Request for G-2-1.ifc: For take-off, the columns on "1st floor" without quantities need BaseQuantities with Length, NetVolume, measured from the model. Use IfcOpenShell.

First a look at what the model holds.

```python
import ifcopenshell
import ifcopenshell.util.element
import ifcopenshell.util.unit

model = ifcopenshell.open("G-2-1.ifc")
print(model.schema)
for unit_type in ("LENGTHUNIT", "AREAUNIT", "VOLUMEUNIT"):
    print(unit_type, ifcopenshell.util.unit.calculate_unit_scale(model, unit_type))
storey = next(s for s in model.by_type("IfcBuildingStorey") if s.Name == "1st floor")
columns = [e for e in ifcopenshell.util.element.get_decomposition(storey) if e.is_a("IfcColumn")]
for e in sorted(columns, key=lambda e: e.id()):
    print(e.id(), e.is_a(), e.Name, list(ifcopenshell.util.element.get_psets(e, qtos_only=True)), sep=" | ")
```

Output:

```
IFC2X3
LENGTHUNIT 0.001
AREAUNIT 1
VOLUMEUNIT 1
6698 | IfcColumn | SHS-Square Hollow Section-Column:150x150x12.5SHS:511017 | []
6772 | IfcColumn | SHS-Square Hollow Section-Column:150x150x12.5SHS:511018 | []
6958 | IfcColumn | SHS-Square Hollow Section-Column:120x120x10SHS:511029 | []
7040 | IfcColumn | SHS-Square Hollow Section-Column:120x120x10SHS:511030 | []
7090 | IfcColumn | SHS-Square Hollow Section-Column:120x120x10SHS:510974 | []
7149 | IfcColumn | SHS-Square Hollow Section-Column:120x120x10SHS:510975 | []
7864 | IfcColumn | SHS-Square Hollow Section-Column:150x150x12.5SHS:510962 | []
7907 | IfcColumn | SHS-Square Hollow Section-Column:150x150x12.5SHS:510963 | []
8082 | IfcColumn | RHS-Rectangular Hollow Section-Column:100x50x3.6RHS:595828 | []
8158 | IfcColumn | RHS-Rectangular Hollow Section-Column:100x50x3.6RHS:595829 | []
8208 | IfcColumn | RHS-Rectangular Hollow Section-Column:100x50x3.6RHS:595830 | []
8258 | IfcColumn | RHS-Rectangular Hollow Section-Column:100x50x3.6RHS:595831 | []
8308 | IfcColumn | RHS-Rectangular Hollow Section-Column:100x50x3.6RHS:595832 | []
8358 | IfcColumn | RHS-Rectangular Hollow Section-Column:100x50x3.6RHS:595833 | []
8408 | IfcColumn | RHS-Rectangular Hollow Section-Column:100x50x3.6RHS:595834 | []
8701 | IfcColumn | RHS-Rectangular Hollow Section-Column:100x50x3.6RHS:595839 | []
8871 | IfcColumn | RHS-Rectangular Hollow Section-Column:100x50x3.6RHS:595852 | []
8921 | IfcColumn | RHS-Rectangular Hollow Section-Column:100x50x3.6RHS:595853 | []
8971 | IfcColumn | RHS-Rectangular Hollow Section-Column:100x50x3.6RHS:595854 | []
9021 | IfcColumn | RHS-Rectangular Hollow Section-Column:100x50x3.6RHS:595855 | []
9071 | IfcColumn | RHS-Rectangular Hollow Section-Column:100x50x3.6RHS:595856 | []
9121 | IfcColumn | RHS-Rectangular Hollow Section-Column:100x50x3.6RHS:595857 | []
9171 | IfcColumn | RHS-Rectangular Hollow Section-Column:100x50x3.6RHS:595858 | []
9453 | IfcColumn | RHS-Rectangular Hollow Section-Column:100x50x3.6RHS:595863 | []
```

```python
import ifcopenshell
import ifcopenshell.api.pset
import ifcopenshell.geom
import ifcopenshell.util.element
import ifcopenshell.util.shape
import ifcopenshell.util.unit

model = ifcopenshell.open("G-2-1.ifc")
unit_scale = ifcopenshell.util.unit.calculate_unit_scale(model)
volume_scale = ifcopenshell.util.unit.calculate_unit_scale(model, "VOLUMEUNIT")
settings = ifcopenshell.geom.settings()

storey = next(s for s in model.by_type("IfcBuildingStorey") if s.Name == "1st floor")
columns = [e for e in ifcopenshell.util.element.get_decomposition(storey) if e.is_a("IfcColumn")]

for e in sorted(columns, key=lambda e: e.id()):
    if ifcopenshell.util.element.get_psets(e, qtos_only=True, should_inherit=False):
        continue
    # Geometry comes back in metres, in the element's own axes.
    shape = ifcopenshell.geom.create_shape(settings, e)
    values = {
        "Length": ifcopenshell.util.shape.get_z(shape.geometry) / unit_scale,
        "NetVolume": ifcopenshell.util.shape.get_volume(shape.geometry) / volume_scale,
    }
    qto = ifcopenshell.api.pset.add_qto(model, product=e, name="BaseQuantities")
    ifcopenshell.api.pset.edit_qto(model, qto=qto, properties=values)
    print(e.id(), {k: round(v, 3) for k, v in values.items()})

model.write("G-2-1-out.ifc")
```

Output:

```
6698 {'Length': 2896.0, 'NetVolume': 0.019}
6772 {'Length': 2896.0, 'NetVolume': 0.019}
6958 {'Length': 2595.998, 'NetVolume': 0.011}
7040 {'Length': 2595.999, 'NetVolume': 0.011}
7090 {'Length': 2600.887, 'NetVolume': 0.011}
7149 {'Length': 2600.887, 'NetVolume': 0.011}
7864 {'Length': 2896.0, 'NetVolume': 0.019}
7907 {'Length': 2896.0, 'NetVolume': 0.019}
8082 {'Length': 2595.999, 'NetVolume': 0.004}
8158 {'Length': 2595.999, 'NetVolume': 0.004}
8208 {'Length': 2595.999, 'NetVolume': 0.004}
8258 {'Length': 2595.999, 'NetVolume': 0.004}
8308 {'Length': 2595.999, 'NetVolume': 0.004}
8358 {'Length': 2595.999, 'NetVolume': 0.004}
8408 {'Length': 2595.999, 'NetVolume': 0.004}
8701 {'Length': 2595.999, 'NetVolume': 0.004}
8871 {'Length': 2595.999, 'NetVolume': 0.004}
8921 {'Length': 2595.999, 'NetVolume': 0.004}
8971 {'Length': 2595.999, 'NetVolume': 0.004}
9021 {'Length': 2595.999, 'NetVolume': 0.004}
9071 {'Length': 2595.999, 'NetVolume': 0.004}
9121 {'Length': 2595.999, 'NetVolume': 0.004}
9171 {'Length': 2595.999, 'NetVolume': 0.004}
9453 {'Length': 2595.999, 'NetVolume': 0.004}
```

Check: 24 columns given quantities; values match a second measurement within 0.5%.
